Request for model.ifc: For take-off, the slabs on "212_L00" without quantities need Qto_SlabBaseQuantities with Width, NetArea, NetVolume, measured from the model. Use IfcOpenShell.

First a look at what the model holds.

```python
import ifcopenshell
import ifcopenshell.util.element
import ifcopenshell.util.unit

model = ifcopenshell.open("model.ifc")
print(model.schema)
for unit_type in ("LENGTHUNIT", "AREAUNIT", "VOLUMEUNIT"):
    print(unit_type, ifcopenshell.util.unit.calculate_unit_scale(model, unit_type))
storey = next(s for s in model.by_type("IfcBuildingStorey") if s.Name == "212_L00")
slabs = [e for e in ifcopenshell.util.element.get_decomposition(storey) if e.is_a("IfcSlab")]
for e in sorted(slabs, key=lambda e: e.id()):
    print(e.id(), e.is_a(), e.Name, list(ifcopenshell.util.element.get_psets(e, qtos_only=True)), sep=" | ")
```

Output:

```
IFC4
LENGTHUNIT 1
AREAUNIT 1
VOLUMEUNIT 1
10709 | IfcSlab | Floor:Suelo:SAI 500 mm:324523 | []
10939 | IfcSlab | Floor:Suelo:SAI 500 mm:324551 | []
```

```python
import ifcopenshell
import ifcopenshell.api.pset
import ifcopenshell.geom
import ifcopenshell.util.element
import ifcopenshell.util.shape
import ifcopenshell.util.unit

model = ifcopenshell.open("model.ifc")
unit_scale = ifcopenshell.util.unit.calculate_unit_scale(model)
area_scale = ifcopenshell.util.unit.calculate_unit_scale(model, "AREAUNIT")
volume_scale = ifcopenshell.util.unit.calculate_unit_scale(model, "VOLUMEUNIT")
settings = ifcopenshell.geom.settings()

storey = next(s for s in model.by_type("IfcBuildingStorey") if s.Name == "212_L00")
slabs = [e for e in ifcopenshell.util.element.get_decomposition(storey) if e.is_a("IfcSlab")]

for e in sorted(slabs, key=lambda e: e.id()):
    if ifcopenshell.util.element.get_psets(e, qtos_only=True, should_inherit=False):
        continue
    # Geometry comes back in metres, in the element's own axes.
    shape = ifcopenshell.geom.create_shape(settings, e)
    values = {
        "Width": ifcopenshell.util.shape.get_z(shape.geometry) / unit_scale,
        "NetArea": ifcopenshell.util.shape.get_footprint_area(shape.geometry) / area_scale,
        "NetVolume": ifcopenshell.util.shape.get_volume(shape.geometry) / volume_scale,
    }
    qto = ifcopenshell.api.pset.add_qto(model, product=e, name="Qto_SlabBaseQuantities")
    ifcopenshell.api.pset.edit_qto(model, qto=qto, properties=values)
    print(e.id(), {k: round(v, 3) for k, v in values.items()})

model.write("model_updated.ifc")
```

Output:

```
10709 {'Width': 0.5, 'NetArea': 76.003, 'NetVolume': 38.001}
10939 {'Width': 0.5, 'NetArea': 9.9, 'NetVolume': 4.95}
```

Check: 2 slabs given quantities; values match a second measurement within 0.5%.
